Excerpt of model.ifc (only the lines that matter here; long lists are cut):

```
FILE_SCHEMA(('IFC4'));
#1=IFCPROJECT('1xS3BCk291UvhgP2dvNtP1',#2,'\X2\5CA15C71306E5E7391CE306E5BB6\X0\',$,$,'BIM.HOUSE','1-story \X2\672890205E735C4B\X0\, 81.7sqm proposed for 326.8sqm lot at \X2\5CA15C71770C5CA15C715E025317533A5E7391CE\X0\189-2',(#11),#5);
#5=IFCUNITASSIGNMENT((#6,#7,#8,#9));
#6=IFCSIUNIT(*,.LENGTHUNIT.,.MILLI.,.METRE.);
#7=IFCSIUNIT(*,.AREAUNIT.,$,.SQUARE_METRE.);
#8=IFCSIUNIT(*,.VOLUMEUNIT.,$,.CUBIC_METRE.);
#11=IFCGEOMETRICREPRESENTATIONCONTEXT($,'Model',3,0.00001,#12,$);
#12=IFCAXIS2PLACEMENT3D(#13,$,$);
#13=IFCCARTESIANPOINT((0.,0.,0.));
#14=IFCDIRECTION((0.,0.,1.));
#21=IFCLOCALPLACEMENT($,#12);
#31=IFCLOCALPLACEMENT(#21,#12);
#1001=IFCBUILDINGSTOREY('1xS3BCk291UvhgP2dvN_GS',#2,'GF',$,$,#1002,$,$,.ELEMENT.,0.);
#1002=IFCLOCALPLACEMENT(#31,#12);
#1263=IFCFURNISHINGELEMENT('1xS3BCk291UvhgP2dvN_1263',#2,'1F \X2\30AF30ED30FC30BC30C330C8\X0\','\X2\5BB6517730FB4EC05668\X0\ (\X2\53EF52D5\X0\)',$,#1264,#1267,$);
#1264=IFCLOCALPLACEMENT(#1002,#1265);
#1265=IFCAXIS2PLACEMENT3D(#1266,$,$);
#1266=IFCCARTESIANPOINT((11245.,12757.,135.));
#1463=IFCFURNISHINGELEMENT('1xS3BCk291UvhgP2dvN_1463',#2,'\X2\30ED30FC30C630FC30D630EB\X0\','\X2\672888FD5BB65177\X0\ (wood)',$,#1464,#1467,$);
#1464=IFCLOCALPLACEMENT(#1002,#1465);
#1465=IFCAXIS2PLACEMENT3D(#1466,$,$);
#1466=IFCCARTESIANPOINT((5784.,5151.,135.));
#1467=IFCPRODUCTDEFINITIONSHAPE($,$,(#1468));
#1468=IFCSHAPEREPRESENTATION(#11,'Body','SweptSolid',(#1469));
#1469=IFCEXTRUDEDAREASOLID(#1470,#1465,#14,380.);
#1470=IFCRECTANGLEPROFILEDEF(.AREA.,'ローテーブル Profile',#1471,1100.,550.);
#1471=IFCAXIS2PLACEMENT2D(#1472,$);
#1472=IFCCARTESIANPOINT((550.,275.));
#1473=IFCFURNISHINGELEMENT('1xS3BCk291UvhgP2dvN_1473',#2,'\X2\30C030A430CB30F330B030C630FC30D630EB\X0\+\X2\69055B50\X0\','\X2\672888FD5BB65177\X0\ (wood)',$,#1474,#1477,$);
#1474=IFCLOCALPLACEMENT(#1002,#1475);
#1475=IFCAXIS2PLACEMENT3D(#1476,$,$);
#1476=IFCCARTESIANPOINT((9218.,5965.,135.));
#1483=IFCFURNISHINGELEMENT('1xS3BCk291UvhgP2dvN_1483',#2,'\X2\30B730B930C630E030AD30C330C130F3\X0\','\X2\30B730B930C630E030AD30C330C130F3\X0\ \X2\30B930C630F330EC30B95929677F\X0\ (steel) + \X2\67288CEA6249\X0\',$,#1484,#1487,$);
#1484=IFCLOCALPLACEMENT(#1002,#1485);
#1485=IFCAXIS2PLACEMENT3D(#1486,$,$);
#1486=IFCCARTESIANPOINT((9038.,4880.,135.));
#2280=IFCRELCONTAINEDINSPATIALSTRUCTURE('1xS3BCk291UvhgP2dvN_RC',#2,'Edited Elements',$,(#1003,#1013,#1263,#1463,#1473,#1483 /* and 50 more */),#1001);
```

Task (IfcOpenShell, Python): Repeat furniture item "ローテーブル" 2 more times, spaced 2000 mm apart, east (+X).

```python
import numpy as np
import ifcopenshell
import ifcopenshell.api.geometry
import ifcopenshell.api.root
import ifcopenshell.util.element
import ifcopenshell.util.placement

model = ifcopenshell.open("model.ifc")


def reuse_history(source, copy):
    """copy_class also copies each property set's owner history, people and application; keep the originals."""
    for rel in copy.IsDefinedBy:
        if rel.is_a("IfcRelDefinesByProperties") and (history := rel.RelatingPropertyDefinition.OwnerHistory):
            rel.RelatingPropertyDefinition.OwnerHistory = source.OwnerHistory
            ifcopenshell.util.element.remove_deep2(model, history)


source = model.by_guid("1xS3BCk291UvhgP2dvN_1463")
base = ifcopenshell.util.placement.get_local_placement(source.ObjectPlacement)
step = np.array([1.0, 0.0, 0.0]) * 2000.0

for i in range(1, 3):
    copy = ifcopenshell.api.root.copy_class(model, product=source)
    copy.Representation = ifcopenshell.util.element.copy_deep(
        model, source.Representation, exclude=["IfcGeometricRepresentationContext", "IfcRepresentationMap"]
    )
    reuse_history(source, copy)
    matrix = base.copy()
    matrix[:3, 3] += i * step
    print("added at", matrix[:3, 3].round(3) + 0.0)
    ifcopenshell.api.geometry.edit_object_placement(model, product=copy, matrix=matrix, is_si=False)

model.write("model-out.ifc")
```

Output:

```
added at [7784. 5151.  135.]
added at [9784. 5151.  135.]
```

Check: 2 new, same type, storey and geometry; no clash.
